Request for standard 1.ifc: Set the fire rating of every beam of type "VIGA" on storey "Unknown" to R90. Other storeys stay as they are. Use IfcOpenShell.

First a look at what the model holds.

```python
import ifcopenshell
import ifcopenshell.util.element

model = ifcopenshell.open("standard 1.ifc")
print(model.schema)
storey = next(s for s in model.by_type("IfcBuildingStorey") if s.Name == "Unknown")
beams = [e for e in ifcopenshell.util.element.get_decomposition(storey) if e.is_a("IfcBeam")]
seen = {}
for e in beams:
    element_type = ifcopenshell.util.element.get_type(e)
    key = (element_type.Name if element_type != e and element_type else None, ifcopenshell.util.element.get_pset(e, "Pset_BeamCommon", "FireRating"))
    seen[key] = seen.get(key, 0) + 1
for (name, value), count in sorted(seen.items(), key=str):
    print(count, "x", name, "|", value)
```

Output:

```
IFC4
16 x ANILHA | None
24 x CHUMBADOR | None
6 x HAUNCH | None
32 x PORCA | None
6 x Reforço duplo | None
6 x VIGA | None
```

```python
import ifcopenshell
import ifcopenshell.api.pset
import ifcopenshell.util.element

model = ifcopenshell.open("standard 1.ifc")

storey = next(s for s in model.by_type("IfcBuildingStorey") if s.Name == "Unknown")
beams = [e for e in ifcopenshell.util.element.get_decomposition(storey) if e.is_a("IfcBeam")]

count = 0
for e in beams:
    element_type = ifcopenshell.util.element.get_type(e)
    if element_type in (None, e) or element_type.Name != "VIGA":
        continue
    found = ifcopenshell.util.element.get_pset(e, "Pset_BeamCommon", should_inherit=False)
    if found:
        pset = model.by_id(found["id"])
        if len(ifcopenshell.util.element.get_elements_by_pset(pset)) > 1:
            pset = ifcopenshell.api.pset.unshare_pset(model, products=[e], pset=pset)[0]
    else:
        pset = ifcopenshell.api.pset.add_pset(model, product=e, name="Pset_BeamCommon")
    ifcopenshell.api.pset.edit_pset(model, pset=pset, properties={"FireRating": "R90"})
    count += 1

print(count, "beams updated")

model.write("standard 1-out.ifc")
```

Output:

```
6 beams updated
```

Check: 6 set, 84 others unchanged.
